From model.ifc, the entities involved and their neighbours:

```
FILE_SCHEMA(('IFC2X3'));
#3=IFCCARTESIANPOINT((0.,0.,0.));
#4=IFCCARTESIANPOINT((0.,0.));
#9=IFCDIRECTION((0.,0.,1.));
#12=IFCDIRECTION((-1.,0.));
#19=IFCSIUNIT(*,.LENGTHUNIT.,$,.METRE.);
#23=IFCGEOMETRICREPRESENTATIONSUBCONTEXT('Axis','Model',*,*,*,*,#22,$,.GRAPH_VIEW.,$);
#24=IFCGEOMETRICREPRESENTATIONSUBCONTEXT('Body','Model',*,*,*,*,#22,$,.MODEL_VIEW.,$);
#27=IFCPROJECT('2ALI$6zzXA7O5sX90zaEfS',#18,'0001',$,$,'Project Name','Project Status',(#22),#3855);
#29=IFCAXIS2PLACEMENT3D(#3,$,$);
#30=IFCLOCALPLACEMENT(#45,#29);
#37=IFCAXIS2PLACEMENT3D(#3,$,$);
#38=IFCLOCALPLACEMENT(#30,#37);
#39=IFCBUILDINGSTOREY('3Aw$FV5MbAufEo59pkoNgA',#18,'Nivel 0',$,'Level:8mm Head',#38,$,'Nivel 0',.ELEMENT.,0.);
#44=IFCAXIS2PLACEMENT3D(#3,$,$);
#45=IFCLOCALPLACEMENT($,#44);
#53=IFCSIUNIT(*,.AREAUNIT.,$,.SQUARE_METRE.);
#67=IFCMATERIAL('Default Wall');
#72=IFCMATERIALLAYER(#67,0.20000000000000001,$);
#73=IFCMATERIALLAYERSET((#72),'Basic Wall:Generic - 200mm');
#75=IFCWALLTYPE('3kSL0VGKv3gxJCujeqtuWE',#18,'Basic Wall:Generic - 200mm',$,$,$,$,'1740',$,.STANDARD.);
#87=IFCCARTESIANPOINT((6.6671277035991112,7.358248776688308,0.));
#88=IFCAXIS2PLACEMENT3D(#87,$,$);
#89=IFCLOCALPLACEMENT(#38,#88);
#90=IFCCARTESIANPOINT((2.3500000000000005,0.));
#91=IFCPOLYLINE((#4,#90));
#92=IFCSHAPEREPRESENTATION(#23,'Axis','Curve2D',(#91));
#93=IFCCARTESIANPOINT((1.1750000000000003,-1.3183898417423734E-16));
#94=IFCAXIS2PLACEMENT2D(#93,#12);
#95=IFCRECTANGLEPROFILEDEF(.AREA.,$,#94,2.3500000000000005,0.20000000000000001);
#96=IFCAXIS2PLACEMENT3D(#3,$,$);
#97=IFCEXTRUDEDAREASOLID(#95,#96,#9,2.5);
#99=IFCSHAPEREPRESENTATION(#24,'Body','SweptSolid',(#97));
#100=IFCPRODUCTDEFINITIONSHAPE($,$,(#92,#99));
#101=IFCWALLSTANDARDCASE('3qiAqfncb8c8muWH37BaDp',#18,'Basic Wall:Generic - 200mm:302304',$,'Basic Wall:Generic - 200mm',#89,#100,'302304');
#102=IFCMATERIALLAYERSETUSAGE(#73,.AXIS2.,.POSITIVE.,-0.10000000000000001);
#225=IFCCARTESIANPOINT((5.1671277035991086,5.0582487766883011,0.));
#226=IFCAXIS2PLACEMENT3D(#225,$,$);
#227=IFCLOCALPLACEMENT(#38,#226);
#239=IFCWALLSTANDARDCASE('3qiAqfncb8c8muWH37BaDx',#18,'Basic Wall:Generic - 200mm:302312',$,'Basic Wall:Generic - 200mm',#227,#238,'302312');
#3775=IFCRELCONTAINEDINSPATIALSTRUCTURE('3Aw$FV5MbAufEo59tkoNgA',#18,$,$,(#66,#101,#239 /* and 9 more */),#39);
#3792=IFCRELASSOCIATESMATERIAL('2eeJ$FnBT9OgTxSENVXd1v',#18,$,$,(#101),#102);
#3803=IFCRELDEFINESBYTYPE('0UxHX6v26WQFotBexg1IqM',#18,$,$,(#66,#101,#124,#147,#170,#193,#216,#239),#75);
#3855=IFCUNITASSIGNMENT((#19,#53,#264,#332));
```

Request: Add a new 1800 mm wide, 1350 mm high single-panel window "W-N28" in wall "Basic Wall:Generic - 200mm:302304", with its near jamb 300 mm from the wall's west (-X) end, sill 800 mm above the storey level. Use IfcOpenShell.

```python
import numpy as np
import ifcopenshell
import ifcopenshell.api.feature
import ifcopenshell.api.geometry
import ifcopenshell.api.root
import ifcopenshell.api.spatial
import ifcopenshell.api.type
import ifcopenshell.geom
import ifcopenshell.util.element
import ifcopenshell.util.placement
import ifcopenshell.util.representation
import ifcopenshell.util.shape
import ifcopenshell.util.unit

model = ifcopenshell.open("model.ifc")
unit_scale = ifcopenshell.util.unit.calculate_unit_scale(model)
settings = ifcopenshell.geom.settings()


def volume(element):
    """Net volume in cubic metres, openings subtracted."""
    shape = ifcopenshell.geom.create_shape(settings, element)
    return ifcopenshell.util.shape.get_volume(shape.geometry)


wall = model.by_guid("3qiAqfncb8c8muWH37BaDp")
storey = ifcopenshell.util.element.get_container(wall, ifc_class="IfcBuildingStorey")
context = ifcopenshell.util.representation.get_context(model, "Model", "Body", "MODEL_VIEW")
before = volume(wall)

width, height, from_end, sill = 1.8, 1.35, 0.3, 0.8  # metres

# The wall runs along its own X axis, and the end named is its -X end.
wall_shape = ifcopenshell.geom.create_shape(settings, wall)
x, y, z = ifcopenshell.util.shape.get_vertices(wall_shape.geometry).T
start = x.min() + from_end
face, thickness = float(y.min()), float(y.max() - y.min())
wall_matrix = ifcopenshell.util.placement.get_local_placement(wall.ObjectPlacement)
level = ifcopenshell.util.placement.get_local_placement(storey.ObjectPlacement)[2, 3]


def in_wall(x, y):
    """Placement at x, y metres in the wall's axes, at sill height."""
    matrix = wall_matrix.copy()
    matrix[:, 3] = wall_matrix @ np.array([x / unit_scale, y / unit_scale, 0.0, 1.0])
    matrix[2, 3] = level + sill / unit_scale
    return matrix


# Opening: a box that overshoots both wall faces by 50 mm.
opening = ifcopenshell.api.root.create_entity(model, ifc_class="IfcOpeningElement")
box = ifcopenshell.api.geometry.add_wall_representation(
    model, context=context, length=width, height=height, thickness=thickness + 0.1
)
ifcopenshell.api.geometry.assign_representation(model, product=opening, representation=box)
ifcopenshell.api.geometry.edit_object_placement(model, product=opening, matrix=in_wall(start, face - 0.05), is_si=False)
ifcopenshell.api.feature.add_feature(model, feature=opening, element=wall)

window = ifcopenshell.api.root.create_entity(model, ifc_class="IfcWindow", name="W-N28")
window.OverallWidth, window.OverallHeight = width / unit_scale, height / unit_scale
body = ifcopenshell.api.geometry.add_window_representation(
    model,
    context=context,
    overall_width=window.OverallWidth,
    overall_height=window.OverallHeight,
    partition_type="SINGLE_PANEL",
)
ifcopenshell.api.geometry.assign_representation(model, product=window, representation=body)
ifcopenshell.api.spatial.assign_container(model, products=[window], relating_structure=storey)
fills = ifcopenshell.api.feature.add_filling(model, opening=opening, element=window)
fills.OwnerHistory = window.OwnerHistory  # required in IFC2X3

# IFC2X3 keeps the operation on the window style.
style = ifcopenshell.api.root.create_entity(model, ifc_class="IfcWindowStyle", name="W-N28")
style.OperationType, style.ConstructionType = "SINGLE_PANEL", "NOTDEFINED"
style.ParameterTakesPrecedence = style.Sizeable = False
ifcopenshell.api.type.assign_type(model, related_objects=[window], relating_type=style)

# Centre the window in the wall's thickness.
ifcopenshell.api.geometry.edit_object_placement(model, product=window, matrix=in_wall(start, face), is_si=False)
window_shape = ifcopenshell.geom.create_shape(settings, window)
depth = ifcopenshell.util.shape.get_vertices(window_shape.geometry)[:, 1]
offset = face + thickness / 2 - (depth.min() + depth.max()) / 2
ifcopenshell.api.geometry.edit_object_placement(model, product=window, matrix=in_wall(start, offset), is_si=False)

after = volume(wall)

print(f"wall volume {before:.3f} -> {after:.3f} m3")

model.write("model_edited.ifc")
```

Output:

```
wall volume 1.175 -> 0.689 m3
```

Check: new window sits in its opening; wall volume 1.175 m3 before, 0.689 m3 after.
